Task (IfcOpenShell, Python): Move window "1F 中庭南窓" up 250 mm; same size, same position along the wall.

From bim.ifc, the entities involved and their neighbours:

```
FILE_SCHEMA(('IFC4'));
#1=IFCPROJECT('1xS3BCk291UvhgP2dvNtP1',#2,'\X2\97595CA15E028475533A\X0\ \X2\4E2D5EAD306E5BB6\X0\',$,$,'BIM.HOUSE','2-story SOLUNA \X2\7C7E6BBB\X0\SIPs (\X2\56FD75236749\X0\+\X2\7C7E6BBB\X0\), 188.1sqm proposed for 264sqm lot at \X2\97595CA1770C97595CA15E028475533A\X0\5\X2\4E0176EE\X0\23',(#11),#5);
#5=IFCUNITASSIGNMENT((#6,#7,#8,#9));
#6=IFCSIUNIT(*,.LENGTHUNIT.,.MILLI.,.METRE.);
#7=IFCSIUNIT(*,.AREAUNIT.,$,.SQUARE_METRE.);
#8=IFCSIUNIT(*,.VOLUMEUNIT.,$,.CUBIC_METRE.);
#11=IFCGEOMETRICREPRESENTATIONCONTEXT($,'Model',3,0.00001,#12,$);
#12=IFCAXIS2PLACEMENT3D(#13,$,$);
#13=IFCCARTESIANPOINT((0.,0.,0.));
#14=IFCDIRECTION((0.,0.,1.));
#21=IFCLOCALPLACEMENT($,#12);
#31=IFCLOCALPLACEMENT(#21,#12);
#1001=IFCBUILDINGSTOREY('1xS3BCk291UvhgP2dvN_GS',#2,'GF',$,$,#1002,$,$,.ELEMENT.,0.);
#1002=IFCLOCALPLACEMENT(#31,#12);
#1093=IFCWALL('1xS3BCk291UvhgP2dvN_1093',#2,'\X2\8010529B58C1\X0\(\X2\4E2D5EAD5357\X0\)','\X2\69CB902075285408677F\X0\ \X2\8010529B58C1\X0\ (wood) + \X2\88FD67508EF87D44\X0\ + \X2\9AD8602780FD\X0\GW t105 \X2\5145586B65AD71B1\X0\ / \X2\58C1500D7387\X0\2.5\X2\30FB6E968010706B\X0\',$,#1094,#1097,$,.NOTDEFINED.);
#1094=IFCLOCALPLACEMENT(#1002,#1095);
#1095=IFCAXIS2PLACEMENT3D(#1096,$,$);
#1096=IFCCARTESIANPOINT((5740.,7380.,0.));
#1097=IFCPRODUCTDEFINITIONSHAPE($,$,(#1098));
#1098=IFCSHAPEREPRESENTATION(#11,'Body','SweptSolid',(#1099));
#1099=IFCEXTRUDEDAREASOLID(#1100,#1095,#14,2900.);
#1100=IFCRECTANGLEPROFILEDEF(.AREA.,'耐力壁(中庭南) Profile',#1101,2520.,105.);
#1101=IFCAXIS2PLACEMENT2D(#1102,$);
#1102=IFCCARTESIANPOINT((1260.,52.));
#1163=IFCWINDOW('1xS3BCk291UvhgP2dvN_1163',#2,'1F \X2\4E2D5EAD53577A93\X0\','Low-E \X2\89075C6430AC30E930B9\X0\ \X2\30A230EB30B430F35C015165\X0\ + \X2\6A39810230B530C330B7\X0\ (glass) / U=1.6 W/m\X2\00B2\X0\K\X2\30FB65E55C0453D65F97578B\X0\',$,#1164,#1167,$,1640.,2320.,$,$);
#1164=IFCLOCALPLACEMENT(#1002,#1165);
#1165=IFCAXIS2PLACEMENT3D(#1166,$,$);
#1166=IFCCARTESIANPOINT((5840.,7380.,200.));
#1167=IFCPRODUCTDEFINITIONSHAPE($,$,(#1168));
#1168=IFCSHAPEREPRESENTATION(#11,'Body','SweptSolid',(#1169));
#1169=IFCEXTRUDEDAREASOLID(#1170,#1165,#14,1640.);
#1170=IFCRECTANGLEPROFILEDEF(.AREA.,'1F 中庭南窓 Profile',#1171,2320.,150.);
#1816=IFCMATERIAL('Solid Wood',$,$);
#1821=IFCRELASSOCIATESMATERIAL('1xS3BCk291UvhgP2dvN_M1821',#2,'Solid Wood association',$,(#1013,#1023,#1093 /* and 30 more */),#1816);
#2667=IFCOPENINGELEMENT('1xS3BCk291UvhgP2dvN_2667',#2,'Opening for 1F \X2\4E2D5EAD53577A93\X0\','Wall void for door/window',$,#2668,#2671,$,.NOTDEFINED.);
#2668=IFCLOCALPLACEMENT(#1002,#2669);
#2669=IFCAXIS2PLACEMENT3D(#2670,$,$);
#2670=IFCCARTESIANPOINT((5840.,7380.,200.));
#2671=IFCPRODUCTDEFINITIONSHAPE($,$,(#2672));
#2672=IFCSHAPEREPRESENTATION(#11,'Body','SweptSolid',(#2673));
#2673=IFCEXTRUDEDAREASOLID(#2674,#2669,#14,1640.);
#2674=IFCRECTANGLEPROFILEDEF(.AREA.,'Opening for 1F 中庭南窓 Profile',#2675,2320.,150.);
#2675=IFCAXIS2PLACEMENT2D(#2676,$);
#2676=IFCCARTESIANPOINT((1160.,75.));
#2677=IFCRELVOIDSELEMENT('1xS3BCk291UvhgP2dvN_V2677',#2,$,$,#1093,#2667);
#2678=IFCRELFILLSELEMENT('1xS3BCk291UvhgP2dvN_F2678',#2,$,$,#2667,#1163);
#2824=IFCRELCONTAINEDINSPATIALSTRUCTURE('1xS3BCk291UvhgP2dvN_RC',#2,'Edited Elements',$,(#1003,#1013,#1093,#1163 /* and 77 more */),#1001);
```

```python
import numpy as np
import ifcopenshell
import ifcopenshell.api.geometry
import ifcopenshell.util.placement
import ifcopenshell.util.unit

model = ifcopenshell.open("bim.ifc")
unit_scale = ifcopenshell.util.unit.calculate_unit_scale(model)

window = model.by_guid("1xS3BCk291UvhgP2dvN_1163")
opening = window.FillsVoids[0].RelatingOpeningElement
dz = 250.0

shift = np.array([0.0, 0.0, dz])
# The window is not placed relative to its opening, so move both.
for product in (opening, window):
    matrix = ifcopenshell.util.placement.get_local_placement(product.ObjectPlacement)
    matrix[:3, 3] += shift
    ifcopenshell.api.geometry.edit_object_placement(model, product=product, matrix=matrix, is_si=False)

print(f"moved by {dz * unit_scale:+.3f} m")

model.write("bim_v2.ifc")
```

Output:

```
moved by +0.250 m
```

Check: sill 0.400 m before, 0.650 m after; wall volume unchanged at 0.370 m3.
